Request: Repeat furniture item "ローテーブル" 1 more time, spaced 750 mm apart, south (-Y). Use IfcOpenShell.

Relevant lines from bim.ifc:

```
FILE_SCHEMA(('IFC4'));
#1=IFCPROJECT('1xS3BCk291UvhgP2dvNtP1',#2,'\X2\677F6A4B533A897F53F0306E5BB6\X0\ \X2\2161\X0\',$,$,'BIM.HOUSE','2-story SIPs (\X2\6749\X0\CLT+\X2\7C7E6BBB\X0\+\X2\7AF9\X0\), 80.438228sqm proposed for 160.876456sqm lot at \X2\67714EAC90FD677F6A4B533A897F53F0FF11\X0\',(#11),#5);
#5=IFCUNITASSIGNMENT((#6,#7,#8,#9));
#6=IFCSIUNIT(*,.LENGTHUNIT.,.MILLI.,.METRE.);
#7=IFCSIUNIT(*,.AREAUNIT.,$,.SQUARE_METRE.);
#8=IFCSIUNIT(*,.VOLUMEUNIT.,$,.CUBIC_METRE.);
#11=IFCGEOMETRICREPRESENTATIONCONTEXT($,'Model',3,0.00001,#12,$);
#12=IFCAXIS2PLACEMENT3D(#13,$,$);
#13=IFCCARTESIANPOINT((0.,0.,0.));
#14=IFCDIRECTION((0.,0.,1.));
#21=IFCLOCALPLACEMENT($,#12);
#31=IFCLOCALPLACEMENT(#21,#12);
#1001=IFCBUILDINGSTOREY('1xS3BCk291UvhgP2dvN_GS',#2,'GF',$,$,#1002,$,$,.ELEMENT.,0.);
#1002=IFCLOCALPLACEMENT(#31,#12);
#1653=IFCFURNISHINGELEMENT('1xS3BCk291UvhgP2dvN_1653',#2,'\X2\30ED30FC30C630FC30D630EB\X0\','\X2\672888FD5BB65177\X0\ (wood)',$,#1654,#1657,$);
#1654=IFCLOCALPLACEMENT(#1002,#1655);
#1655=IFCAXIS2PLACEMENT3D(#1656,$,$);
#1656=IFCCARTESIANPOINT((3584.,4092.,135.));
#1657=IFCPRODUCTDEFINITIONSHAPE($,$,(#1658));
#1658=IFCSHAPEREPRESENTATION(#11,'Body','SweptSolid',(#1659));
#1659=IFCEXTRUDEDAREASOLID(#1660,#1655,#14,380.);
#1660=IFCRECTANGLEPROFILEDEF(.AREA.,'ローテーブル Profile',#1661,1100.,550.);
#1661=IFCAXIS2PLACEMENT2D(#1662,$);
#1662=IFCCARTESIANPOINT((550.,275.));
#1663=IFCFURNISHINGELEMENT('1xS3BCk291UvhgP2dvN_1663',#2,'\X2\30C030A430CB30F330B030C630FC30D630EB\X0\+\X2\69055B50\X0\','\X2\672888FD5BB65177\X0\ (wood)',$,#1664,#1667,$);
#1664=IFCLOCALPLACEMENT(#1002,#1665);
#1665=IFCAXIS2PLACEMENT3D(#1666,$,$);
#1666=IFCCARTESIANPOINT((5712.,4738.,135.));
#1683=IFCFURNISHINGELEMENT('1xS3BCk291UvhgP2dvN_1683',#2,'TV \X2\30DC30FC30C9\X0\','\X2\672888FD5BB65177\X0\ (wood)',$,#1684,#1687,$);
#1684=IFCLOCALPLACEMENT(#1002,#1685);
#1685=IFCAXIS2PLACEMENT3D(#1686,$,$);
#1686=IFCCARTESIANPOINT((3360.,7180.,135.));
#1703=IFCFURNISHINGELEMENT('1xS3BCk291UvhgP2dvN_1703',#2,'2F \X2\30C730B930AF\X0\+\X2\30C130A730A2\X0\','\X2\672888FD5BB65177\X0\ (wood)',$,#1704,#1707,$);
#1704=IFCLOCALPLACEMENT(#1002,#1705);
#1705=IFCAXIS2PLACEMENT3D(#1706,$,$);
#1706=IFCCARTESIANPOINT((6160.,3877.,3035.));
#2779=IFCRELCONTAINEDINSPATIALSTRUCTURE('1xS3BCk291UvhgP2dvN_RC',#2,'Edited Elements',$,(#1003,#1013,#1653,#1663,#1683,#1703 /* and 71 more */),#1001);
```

```python
import numpy as np
import ifcopenshell
import ifcopenshell.api.geometry
import ifcopenshell.api.root
import ifcopenshell.util.element
import ifcopenshell.util.placement
import ifcopenshell.util.unit

model = ifcopenshell.open("bim.ifc")
unit_scale = ifcopenshell.util.unit.calculate_unit_scale(model)


def reuse_history(source, copy):
    """copy_class also copies each property set's owner history, people and application; keep the originals."""
    for rel in copy.IsDefinedBy:
        if rel.is_a("IfcRelDefinesByProperties") and (history := rel.RelatingPropertyDefinition.OwnerHistory):
            rel.RelatingPropertyDefinition.OwnerHistory = source.OwnerHistory
            ifcopenshell.util.element.remove_deep2(model, history)


source = model.by_id(1653)
base = ifcopenshell.util.placement.get_local_placement(source.ObjectPlacement)
step = np.array([0.0, -1.0, 0.0]) * 0.75 / unit_scale

for i in range(1, 2):
    copy = ifcopenshell.api.root.copy_class(model, product=source)
    copy.Representation = ifcopenshell.util.element.copy_deep(
        model, source.Representation, exclude=["IfcGeometricRepresentationContext", "IfcRepresentationMap"]
    )
    reuse_history(source, copy)
    matrix = base.copy()
    matrix[:3, 3] += i * step
    print("added at", matrix[:3, 3].round(3) + 0.0)
    ifcopenshell.api.geometry.edit_object_placement(model, product=copy, matrix=matrix, is_si=False)

model.write("bim_edited.ifc")
```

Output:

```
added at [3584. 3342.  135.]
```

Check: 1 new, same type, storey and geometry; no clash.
